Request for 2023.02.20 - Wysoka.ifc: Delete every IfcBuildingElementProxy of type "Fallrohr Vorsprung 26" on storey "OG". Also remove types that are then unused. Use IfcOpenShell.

First a look at what the model holds.

```python
import ifcopenshell
import ifcopenshell.util.element

model = ifcopenshell.open("2023.02.20 - Wysoka.ifc")
print(model.schema)
storey = next(s for s in model.by_type("IfcBuildingStorey") if s.Name == "OG")
proxies = [e for e in ifcopenshell.util.element.get_decomposition(storey) if e.is_a("IfcBuildingElementProxy")]
seen = {}
for e in proxies:
    element_type = ifcopenshell.util.element.get_type(e)
    name = element_type.Name if element_type not in (None, e) else None
    seen[name] = seen.get(name, 0) + 1
for name, count in sorted(seen.items(), key=str):
    print(count, "x", name)
```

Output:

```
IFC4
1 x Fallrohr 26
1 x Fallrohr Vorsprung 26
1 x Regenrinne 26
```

```python
import ifcopenshell
import ifcopenshell.api.root
import ifcopenshell.util.element

model = ifcopenshell.open("2023.02.20 - Wysoka.ifc")

storey = next(s for s in model.by_type("IfcBuildingStorey") if s.Name == "OG")
proxies = [e for e in ifcopenshell.util.element.get_decomposition(storey) if e.is_a("IfcBuildingElementProxy")]
targets = [e for e in proxies if (t := ifcopenshell.util.element.get_type(e)) not in (None, e) and t.Name == "Fallrohr Vorsprung 26"]
types = {ifcopenshell.util.element.get_type(e) for e in targets} - {None, *targets}

for e in targets:
    ifcopenshell.api.root.remove_product(model, product=e)
print(len(targets), "removed")

unused = [t for t in types if not ifcopenshell.util.element.get_types(t)]
for t in unused:
    ifcopenshell.api.root.remove_product(model, product=t)
print(len(unused), "unused types removed")

model.write("2023.02.20 - Wysoka_rev.ifc")
```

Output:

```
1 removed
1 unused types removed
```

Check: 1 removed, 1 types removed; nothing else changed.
